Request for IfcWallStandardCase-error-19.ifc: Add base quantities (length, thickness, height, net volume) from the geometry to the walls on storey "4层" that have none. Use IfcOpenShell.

First a look at what the model holds.

```python
import ifcopenshell
import ifcopenshell.util.element
import ifcopenshell.util.unit

model = ifcopenshell.open("IfcWallStandardCase-error-19.ifc")
print(model.schema)
for unit_type in ("LENGTHUNIT", "AREAUNIT", "VOLUMEUNIT"):
    print(unit_type, ifcopenshell.util.unit.calculate_unit_scale(model, unit_type))
storey = next(s for s in model.by_type("IfcBuildingStorey") if s.Name == "4层")
walls = [e for e in ifcopenshell.util.element.get_decomposition(storey) if e.is_a("IfcWall")]
for e in sorted(walls, key=lambda e: e.id()):
    print(e.id(), e.is_a(), e.Name, list(ifcopenshell.util.element.get_psets(e, qtos_only=True)), sep=" | ")
```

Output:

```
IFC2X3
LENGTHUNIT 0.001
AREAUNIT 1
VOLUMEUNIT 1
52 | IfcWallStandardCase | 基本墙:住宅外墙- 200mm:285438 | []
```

```python
import ifcopenshell
import ifcopenshell.api.pset
import ifcopenshell.geom
import ifcopenshell.util.element
import ifcopenshell.util.shape
import ifcopenshell.util.unit

model = ifcopenshell.open("IfcWallStandardCase-error-19.ifc")
unit_scale = ifcopenshell.util.unit.calculate_unit_scale(model)
volume_scale = ifcopenshell.util.unit.calculate_unit_scale(model, "VOLUMEUNIT")
settings = ifcopenshell.geom.settings()

storey = next(s for s in model.by_type("IfcBuildingStorey") if s.Name == "4层")
walls = [e for e in ifcopenshell.util.element.get_decomposition(storey) if e.is_a("IfcWall")]

for e in sorted(walls, key=lambda e: e.id()):
    if ifcopenshell.util.element.get_psets(e, qtos_only=True, should_inherit=False):
        continue
    # Geometry comes back in metres, in the element's own axes.
    shape = ifcopenshell.geom.create_shape(settings, e)
    values = {
        "Length": ifcopenshell.util.shape.get_x(shape.geometry) / unit_scale,
        "Width": ifcopenshell.util.shape.get_y(shape.geometry) / unit_scale,
        "Height": ifcopenshell.util.shape.get_z(shape.geometry) / unit_scale,
        "NetVolume": ifcopenshell.util.shape.get_volume(shape.geometry) / volume_scale,
    }
    qto = ifcopenshell.api.pset.add_qto(model, product=e, name="BaseQuantities")
    ifcopenshell.api.pset.edit_qto(model, qto=qto, properties=values)
    print(e.id(), {k: round(v, 3) for k, v in values.items()})

model.write("IfcWallStandardCase-error-19_rev.ifc")
```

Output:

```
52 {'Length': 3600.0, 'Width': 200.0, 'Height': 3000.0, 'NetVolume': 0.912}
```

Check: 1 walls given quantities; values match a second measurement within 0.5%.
